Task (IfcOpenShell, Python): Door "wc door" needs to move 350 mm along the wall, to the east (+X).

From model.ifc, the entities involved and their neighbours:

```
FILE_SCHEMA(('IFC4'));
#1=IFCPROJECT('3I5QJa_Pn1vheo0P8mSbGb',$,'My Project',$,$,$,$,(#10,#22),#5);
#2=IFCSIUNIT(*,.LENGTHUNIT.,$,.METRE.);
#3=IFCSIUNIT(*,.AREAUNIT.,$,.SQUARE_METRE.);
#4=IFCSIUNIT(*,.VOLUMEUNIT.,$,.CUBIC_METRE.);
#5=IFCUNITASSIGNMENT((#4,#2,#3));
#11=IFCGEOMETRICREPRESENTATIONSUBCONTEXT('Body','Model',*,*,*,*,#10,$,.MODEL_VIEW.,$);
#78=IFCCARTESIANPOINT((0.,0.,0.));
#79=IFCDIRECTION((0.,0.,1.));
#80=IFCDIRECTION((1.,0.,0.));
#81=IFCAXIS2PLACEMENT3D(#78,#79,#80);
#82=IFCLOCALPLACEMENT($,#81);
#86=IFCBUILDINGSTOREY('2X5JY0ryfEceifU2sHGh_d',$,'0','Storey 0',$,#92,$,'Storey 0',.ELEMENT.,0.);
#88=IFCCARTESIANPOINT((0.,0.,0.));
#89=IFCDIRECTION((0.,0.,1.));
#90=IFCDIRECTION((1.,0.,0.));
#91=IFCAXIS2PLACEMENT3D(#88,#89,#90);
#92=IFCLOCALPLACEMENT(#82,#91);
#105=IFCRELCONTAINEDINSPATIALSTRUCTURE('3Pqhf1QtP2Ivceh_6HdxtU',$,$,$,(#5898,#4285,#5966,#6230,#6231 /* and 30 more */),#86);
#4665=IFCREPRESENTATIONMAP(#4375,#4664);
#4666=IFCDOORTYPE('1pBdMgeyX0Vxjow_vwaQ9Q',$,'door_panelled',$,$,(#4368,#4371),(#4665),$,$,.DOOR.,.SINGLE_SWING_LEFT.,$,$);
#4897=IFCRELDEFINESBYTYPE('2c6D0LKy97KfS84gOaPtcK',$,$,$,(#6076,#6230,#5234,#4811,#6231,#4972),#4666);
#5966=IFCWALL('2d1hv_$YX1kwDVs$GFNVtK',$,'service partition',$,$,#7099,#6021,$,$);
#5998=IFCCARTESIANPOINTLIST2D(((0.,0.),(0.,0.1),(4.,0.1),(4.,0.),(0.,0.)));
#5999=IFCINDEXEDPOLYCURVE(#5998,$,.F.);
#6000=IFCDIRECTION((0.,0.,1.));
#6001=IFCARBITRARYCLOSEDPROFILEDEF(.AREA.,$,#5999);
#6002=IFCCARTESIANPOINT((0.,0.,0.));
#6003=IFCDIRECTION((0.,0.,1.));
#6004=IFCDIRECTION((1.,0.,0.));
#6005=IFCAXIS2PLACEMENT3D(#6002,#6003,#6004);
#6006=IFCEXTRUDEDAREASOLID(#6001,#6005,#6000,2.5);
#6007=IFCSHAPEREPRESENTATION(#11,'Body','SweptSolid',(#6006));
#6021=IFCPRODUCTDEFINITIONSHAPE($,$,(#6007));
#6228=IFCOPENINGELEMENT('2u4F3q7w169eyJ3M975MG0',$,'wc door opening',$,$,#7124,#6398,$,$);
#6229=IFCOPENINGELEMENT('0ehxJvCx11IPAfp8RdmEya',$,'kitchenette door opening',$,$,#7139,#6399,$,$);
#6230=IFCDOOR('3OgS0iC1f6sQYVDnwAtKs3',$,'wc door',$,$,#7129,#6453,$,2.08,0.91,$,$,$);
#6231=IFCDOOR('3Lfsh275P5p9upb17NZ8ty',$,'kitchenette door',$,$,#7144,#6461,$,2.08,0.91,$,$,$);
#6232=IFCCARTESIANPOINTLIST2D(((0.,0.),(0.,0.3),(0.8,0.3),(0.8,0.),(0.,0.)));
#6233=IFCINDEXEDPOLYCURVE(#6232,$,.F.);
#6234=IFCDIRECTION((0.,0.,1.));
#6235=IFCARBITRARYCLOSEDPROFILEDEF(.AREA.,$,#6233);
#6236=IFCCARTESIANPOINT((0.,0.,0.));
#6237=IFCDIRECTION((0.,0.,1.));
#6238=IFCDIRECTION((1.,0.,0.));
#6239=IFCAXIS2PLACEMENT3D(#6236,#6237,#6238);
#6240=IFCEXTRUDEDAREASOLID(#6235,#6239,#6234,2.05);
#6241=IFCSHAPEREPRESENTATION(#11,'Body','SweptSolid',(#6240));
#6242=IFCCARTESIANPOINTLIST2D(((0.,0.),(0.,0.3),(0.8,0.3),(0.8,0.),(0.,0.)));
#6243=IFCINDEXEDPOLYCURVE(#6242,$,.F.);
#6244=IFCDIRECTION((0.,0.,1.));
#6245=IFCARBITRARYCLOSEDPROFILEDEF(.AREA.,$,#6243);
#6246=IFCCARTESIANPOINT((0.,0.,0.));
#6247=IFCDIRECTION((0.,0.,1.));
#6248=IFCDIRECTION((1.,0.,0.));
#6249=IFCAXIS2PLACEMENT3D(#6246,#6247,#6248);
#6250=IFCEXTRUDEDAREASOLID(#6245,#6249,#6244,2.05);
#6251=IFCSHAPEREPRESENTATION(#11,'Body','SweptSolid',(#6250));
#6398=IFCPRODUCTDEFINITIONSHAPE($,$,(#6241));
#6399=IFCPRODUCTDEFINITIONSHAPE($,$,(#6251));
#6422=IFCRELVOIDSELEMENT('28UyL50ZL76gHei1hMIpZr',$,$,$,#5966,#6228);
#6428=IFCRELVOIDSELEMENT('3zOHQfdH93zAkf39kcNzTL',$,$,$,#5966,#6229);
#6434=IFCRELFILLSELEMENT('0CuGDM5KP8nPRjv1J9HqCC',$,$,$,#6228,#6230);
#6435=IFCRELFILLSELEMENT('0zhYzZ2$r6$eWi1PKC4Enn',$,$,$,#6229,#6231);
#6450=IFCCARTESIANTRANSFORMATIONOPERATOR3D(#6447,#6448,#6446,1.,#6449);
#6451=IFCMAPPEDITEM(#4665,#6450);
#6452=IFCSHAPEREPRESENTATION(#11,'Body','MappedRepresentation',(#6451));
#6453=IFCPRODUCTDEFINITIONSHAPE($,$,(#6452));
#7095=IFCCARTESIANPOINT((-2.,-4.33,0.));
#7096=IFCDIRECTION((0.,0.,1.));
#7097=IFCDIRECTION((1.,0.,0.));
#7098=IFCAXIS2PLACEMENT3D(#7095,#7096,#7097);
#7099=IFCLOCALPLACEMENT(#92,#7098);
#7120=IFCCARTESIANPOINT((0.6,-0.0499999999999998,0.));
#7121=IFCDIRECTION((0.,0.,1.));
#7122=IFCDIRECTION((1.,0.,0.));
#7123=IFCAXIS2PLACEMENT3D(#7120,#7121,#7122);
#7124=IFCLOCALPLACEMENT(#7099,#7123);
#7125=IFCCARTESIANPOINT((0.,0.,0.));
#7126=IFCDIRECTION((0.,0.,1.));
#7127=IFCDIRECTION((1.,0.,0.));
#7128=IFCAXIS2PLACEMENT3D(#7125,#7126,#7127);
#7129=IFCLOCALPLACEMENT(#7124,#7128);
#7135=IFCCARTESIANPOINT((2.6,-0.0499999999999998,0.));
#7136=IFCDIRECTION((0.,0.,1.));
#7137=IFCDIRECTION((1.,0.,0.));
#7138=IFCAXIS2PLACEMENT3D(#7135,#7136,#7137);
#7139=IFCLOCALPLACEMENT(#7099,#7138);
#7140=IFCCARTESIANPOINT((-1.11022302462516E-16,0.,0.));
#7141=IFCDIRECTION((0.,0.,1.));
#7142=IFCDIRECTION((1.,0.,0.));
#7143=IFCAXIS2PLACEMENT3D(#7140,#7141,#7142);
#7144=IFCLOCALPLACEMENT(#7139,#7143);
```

```python
import ifcopenshell
import ifcopenshell.api.geometry
import ifcopenshell.util.placement
import ifcopenshell.util.unit

model = ifcopenshell.open("model.ifc")
unit_scale = ifcopenshell.util.unit.calculate_unit_scale(model)

door = model.by_guid("3OgS0iC1f6sQYVDnwAtKs3")
opening = door.FillsVoids[0].RelatingOpeningElement
wall = opening.VoidsElements[0].RelatingBuildingElement

wall_matrix = ifcopenshell.util.placement.get_local_placement(wall.ObjectPlacement)
shift = wall_matrix[:3, 0] * 0.35 / unit_scale
before = ifcopenshell.util.placement.get_local_placement(door.ObjectPlacement)[:3, 3].copy()

# The door is placed relative to its opening, so it follows when the opening moves.
matrix = ifcopenshell.util.placement.get_local_placement(opening.ObjectPlacement)
matrix[:3, 3] += shift
ifcopenshell.api.geometry.edit_object_placement(
    model, product=opening, matrix=matrix, is_si=False, should_transform_children=True
)

after = ifcopenshell.util.placement.get_local_placement(door.ObjectPlacement)[:3, 3]
print("door moved by", (after - before).round(3) + 0.0)

model.write("model-out.ifc")
```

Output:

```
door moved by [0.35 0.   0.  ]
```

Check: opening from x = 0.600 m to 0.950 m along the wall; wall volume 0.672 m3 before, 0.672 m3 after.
